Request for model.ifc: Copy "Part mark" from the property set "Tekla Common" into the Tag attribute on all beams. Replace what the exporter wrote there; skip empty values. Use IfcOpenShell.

First a look at what the model holds.

```python
import ifcopenshell
import ifcopenshell.util.element

model = ifcopenshell.open("model.ifc")
print(model.schema)
beams = model.by_type("IfcBeam")
print(len(beams), "beams")
for e in beams[:8]:
    source = ifcopenshell.util.element.get_pset(e, "Tekla Common", "Part mark")
    target = e.Tag
    print(e.id(), repr(source), repr(target), sep=" | ")
```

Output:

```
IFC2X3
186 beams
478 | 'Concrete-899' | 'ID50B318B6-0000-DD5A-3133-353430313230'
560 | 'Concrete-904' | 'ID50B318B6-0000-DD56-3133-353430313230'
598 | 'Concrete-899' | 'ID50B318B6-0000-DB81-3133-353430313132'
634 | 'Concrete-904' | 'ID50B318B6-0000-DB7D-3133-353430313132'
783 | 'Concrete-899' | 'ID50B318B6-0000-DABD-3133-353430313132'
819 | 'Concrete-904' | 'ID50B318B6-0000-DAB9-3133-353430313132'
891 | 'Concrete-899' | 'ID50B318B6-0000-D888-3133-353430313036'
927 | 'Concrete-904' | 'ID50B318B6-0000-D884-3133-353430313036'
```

```python
import ifcopenshell
import ifcopenshell.util.element

model = ifcopenshell.open("model.ifc")

count = 0
for e in model.by_type("IfcBeam"):
    value = ifcopenshell.util.element.get_pset(e, "Tekla Common", "Part mark")
    current = e.Tag
    if not value or not value.strip() or current == value:
        continue
    e.Tag = value
    count += 1

print(count, "beams updated")

model.write("model_rev.ifc")
```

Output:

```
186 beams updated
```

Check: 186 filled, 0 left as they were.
